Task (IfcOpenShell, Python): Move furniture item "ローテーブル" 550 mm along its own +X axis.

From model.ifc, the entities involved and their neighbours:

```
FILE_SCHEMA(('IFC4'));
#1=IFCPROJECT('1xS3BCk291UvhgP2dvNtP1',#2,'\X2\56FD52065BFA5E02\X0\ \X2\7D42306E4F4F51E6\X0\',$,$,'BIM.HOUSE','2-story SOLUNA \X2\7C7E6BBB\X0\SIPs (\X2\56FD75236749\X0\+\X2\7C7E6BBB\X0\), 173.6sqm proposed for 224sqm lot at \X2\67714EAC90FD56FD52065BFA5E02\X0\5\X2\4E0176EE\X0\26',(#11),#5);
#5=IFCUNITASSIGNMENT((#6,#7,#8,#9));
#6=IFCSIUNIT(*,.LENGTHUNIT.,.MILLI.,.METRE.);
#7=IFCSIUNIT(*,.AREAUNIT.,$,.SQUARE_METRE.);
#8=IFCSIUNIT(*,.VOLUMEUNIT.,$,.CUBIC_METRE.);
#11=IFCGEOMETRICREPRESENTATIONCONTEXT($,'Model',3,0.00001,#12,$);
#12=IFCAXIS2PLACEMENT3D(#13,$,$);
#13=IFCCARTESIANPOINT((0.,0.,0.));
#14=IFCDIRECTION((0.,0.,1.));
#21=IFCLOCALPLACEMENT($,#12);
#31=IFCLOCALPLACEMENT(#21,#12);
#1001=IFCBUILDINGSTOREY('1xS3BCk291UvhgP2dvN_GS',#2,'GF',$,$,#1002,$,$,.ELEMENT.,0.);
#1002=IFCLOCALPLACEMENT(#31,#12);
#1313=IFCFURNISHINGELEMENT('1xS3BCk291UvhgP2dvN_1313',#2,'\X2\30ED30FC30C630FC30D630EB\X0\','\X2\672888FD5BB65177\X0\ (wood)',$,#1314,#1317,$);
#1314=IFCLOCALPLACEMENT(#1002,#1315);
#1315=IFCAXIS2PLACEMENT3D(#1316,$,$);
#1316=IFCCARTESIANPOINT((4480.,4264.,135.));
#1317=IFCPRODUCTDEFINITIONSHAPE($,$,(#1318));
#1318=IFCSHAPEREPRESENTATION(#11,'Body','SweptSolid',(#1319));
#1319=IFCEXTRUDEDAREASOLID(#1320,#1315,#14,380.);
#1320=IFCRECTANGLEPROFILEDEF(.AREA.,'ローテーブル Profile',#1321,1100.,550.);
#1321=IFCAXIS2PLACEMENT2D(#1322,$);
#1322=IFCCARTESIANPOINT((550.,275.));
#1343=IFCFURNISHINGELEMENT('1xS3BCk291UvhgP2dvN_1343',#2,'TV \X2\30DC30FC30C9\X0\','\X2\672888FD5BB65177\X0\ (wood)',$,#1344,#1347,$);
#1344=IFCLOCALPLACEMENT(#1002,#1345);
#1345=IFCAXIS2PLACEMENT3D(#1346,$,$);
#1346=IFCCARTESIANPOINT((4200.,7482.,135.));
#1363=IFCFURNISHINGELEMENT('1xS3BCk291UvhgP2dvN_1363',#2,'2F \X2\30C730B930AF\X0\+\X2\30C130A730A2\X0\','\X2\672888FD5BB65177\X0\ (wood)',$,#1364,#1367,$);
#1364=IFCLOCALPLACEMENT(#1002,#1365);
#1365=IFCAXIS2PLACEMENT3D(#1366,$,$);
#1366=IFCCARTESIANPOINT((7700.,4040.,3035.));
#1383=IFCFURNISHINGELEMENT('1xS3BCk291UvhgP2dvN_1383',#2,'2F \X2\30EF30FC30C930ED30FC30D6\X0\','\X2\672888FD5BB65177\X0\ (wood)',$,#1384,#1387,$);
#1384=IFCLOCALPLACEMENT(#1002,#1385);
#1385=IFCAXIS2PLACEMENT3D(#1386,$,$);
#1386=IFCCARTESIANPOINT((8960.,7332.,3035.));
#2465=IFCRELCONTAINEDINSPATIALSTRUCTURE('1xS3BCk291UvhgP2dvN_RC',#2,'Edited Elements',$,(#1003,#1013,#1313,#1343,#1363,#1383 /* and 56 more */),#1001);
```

```python
import ifcopenshell
import ifcopenshell.api.geometry
import ifcopenshell.util.placement

model = ifcopenshell.open("model.ifc")

item = model.by_id(1313)
matrix = ifcopenshell.util.placement.get_local_placement(item.ObjectPlacement)
matrix[:3, 3] += matrix[:3, 0] * 550.0
ifcopenshell.api.geometry.edit_object_placement(model, product=item, matrix=matrix, is_si=False)

print(ifcopenshell.util.placement.get_local_placement(item.ObjectPlacement).round(3) + 0.0)

model.write("model_updated.ifc")
```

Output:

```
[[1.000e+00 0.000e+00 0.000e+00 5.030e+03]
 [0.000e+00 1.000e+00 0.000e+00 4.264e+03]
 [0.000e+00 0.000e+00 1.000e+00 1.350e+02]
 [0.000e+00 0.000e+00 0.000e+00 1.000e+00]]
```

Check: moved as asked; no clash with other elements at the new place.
